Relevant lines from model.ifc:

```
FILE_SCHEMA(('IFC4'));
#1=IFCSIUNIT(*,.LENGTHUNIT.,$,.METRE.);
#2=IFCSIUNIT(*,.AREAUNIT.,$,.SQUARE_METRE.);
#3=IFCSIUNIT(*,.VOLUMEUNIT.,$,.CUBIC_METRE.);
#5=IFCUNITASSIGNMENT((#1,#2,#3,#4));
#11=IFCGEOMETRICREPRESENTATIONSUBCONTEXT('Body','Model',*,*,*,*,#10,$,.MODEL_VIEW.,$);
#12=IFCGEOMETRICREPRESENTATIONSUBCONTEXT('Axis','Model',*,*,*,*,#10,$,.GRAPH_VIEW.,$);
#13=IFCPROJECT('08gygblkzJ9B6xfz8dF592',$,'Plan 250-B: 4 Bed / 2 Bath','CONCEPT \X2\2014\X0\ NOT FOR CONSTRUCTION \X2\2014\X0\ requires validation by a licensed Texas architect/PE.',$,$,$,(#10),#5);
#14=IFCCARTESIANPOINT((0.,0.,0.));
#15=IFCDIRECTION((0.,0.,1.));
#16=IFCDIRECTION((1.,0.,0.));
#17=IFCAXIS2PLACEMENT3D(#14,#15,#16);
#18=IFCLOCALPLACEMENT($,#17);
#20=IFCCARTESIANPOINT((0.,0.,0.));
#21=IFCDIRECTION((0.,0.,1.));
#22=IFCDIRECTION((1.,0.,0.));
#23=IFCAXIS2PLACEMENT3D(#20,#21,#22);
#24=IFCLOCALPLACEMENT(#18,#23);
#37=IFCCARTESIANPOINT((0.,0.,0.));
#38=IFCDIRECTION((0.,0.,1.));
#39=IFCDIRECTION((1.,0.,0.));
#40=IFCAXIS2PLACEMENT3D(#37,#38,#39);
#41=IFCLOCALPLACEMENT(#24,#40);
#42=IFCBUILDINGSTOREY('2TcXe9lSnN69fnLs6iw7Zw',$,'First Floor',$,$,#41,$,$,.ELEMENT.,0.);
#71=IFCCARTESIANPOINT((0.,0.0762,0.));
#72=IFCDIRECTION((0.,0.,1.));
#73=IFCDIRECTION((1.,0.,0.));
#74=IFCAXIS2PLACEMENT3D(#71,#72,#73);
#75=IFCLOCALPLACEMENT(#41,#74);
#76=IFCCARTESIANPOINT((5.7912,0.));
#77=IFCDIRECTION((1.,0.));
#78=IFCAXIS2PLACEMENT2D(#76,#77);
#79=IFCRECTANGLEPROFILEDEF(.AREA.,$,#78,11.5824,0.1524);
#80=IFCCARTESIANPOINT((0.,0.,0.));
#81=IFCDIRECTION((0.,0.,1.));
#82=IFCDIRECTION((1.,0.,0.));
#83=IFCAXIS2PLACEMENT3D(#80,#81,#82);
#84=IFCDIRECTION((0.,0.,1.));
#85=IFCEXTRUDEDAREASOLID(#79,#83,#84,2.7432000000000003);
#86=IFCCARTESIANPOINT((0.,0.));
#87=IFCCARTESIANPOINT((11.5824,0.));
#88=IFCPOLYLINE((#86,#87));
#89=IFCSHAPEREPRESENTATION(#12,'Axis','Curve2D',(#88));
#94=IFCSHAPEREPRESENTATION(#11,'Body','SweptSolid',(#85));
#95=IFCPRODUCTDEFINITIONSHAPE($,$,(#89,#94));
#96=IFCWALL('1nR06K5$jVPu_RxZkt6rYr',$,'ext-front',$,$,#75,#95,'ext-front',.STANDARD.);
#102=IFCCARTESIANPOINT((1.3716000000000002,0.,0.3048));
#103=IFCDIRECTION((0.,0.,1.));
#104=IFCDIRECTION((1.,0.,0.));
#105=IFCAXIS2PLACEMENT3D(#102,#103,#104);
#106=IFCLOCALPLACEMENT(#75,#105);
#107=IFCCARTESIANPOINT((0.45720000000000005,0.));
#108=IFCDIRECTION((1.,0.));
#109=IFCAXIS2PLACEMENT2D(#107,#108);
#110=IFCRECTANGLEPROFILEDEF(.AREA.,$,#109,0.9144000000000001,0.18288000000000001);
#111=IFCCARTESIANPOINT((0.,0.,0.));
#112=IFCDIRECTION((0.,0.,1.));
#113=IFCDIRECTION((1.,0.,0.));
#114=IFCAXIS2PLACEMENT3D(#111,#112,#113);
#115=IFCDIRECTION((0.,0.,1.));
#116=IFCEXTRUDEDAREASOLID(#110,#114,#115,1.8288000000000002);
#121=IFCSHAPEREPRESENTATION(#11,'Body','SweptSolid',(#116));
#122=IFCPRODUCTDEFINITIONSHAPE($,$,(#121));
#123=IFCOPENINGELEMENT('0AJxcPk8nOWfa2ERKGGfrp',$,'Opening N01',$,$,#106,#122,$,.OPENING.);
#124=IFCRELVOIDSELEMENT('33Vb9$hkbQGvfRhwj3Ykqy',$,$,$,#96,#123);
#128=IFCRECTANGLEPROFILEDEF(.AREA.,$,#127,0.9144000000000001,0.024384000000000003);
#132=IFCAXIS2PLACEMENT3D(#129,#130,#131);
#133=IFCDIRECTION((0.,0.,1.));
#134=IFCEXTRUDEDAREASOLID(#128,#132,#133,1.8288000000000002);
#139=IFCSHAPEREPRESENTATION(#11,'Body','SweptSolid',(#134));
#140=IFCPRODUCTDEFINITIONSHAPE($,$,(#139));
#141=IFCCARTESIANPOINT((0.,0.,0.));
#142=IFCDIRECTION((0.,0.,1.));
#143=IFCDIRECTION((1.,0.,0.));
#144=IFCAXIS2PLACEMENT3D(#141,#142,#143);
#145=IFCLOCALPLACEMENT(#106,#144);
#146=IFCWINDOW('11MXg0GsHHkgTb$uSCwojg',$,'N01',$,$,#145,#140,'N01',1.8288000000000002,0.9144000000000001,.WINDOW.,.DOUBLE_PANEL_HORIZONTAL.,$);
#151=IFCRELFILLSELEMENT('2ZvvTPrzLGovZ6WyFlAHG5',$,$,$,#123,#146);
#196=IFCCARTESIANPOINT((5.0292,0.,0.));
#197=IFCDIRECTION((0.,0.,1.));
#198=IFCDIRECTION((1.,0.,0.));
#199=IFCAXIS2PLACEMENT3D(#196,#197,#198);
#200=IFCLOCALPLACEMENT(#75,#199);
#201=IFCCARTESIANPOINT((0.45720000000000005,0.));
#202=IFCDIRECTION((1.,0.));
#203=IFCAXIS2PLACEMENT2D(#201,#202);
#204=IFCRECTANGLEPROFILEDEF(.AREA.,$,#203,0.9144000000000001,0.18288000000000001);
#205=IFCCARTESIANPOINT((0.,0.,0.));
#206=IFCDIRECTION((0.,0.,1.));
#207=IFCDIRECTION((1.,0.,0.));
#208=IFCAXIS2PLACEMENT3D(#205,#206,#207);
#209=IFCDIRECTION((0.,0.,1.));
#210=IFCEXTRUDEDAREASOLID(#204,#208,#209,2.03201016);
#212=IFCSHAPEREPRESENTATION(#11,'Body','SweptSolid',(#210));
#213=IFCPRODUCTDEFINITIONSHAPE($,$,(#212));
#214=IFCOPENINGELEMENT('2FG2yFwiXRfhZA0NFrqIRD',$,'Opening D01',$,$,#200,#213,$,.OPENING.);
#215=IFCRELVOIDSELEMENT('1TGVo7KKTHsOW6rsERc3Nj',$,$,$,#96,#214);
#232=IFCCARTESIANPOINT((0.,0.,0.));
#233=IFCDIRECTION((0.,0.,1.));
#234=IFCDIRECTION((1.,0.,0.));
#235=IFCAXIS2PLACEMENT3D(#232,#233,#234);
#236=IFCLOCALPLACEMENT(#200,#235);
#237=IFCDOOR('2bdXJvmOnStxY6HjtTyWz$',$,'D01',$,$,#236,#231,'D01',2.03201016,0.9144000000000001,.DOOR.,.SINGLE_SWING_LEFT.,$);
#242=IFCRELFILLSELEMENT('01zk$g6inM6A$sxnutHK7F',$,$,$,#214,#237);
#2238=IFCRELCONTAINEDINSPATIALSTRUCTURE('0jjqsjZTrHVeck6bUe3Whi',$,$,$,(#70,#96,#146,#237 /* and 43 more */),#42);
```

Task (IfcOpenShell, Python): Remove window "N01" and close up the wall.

```python
import ifcopenshell
import ifcopenshell.api.feature
import ifcopenshell.api.root
import ifcopenshell.geom
import ifcopenshell.util.shape

model = ifcopenshell.open("model.ifc")
settings = ifcopenshell.geom.settings()


def volume(element):
    """Net volume in cubic metres, openings subtracted."""
    shape = ifcopenshell.geom.create_shape(settings, element)
    return ifcopenshell.util.shape.get_volume(shape.geometry)


window = model.by_id(146)
opening = window.FillsVoids[0].RelatingOpeningElement
wall = opening.VoidsElements[0].RelatingBuildingElement
before = volume(wall)

ifcopenshell.api.root.remove_product(model, product=window)
ifcopenshell.api.feature.remove_feature(model, feature=opening)

after = volume(wall)

print(f"wall volume {before:.3f} -> {after:.3f} m3")

model.write("model-out.ifc")
```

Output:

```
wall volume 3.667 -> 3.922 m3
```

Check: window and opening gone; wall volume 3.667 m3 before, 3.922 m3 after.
